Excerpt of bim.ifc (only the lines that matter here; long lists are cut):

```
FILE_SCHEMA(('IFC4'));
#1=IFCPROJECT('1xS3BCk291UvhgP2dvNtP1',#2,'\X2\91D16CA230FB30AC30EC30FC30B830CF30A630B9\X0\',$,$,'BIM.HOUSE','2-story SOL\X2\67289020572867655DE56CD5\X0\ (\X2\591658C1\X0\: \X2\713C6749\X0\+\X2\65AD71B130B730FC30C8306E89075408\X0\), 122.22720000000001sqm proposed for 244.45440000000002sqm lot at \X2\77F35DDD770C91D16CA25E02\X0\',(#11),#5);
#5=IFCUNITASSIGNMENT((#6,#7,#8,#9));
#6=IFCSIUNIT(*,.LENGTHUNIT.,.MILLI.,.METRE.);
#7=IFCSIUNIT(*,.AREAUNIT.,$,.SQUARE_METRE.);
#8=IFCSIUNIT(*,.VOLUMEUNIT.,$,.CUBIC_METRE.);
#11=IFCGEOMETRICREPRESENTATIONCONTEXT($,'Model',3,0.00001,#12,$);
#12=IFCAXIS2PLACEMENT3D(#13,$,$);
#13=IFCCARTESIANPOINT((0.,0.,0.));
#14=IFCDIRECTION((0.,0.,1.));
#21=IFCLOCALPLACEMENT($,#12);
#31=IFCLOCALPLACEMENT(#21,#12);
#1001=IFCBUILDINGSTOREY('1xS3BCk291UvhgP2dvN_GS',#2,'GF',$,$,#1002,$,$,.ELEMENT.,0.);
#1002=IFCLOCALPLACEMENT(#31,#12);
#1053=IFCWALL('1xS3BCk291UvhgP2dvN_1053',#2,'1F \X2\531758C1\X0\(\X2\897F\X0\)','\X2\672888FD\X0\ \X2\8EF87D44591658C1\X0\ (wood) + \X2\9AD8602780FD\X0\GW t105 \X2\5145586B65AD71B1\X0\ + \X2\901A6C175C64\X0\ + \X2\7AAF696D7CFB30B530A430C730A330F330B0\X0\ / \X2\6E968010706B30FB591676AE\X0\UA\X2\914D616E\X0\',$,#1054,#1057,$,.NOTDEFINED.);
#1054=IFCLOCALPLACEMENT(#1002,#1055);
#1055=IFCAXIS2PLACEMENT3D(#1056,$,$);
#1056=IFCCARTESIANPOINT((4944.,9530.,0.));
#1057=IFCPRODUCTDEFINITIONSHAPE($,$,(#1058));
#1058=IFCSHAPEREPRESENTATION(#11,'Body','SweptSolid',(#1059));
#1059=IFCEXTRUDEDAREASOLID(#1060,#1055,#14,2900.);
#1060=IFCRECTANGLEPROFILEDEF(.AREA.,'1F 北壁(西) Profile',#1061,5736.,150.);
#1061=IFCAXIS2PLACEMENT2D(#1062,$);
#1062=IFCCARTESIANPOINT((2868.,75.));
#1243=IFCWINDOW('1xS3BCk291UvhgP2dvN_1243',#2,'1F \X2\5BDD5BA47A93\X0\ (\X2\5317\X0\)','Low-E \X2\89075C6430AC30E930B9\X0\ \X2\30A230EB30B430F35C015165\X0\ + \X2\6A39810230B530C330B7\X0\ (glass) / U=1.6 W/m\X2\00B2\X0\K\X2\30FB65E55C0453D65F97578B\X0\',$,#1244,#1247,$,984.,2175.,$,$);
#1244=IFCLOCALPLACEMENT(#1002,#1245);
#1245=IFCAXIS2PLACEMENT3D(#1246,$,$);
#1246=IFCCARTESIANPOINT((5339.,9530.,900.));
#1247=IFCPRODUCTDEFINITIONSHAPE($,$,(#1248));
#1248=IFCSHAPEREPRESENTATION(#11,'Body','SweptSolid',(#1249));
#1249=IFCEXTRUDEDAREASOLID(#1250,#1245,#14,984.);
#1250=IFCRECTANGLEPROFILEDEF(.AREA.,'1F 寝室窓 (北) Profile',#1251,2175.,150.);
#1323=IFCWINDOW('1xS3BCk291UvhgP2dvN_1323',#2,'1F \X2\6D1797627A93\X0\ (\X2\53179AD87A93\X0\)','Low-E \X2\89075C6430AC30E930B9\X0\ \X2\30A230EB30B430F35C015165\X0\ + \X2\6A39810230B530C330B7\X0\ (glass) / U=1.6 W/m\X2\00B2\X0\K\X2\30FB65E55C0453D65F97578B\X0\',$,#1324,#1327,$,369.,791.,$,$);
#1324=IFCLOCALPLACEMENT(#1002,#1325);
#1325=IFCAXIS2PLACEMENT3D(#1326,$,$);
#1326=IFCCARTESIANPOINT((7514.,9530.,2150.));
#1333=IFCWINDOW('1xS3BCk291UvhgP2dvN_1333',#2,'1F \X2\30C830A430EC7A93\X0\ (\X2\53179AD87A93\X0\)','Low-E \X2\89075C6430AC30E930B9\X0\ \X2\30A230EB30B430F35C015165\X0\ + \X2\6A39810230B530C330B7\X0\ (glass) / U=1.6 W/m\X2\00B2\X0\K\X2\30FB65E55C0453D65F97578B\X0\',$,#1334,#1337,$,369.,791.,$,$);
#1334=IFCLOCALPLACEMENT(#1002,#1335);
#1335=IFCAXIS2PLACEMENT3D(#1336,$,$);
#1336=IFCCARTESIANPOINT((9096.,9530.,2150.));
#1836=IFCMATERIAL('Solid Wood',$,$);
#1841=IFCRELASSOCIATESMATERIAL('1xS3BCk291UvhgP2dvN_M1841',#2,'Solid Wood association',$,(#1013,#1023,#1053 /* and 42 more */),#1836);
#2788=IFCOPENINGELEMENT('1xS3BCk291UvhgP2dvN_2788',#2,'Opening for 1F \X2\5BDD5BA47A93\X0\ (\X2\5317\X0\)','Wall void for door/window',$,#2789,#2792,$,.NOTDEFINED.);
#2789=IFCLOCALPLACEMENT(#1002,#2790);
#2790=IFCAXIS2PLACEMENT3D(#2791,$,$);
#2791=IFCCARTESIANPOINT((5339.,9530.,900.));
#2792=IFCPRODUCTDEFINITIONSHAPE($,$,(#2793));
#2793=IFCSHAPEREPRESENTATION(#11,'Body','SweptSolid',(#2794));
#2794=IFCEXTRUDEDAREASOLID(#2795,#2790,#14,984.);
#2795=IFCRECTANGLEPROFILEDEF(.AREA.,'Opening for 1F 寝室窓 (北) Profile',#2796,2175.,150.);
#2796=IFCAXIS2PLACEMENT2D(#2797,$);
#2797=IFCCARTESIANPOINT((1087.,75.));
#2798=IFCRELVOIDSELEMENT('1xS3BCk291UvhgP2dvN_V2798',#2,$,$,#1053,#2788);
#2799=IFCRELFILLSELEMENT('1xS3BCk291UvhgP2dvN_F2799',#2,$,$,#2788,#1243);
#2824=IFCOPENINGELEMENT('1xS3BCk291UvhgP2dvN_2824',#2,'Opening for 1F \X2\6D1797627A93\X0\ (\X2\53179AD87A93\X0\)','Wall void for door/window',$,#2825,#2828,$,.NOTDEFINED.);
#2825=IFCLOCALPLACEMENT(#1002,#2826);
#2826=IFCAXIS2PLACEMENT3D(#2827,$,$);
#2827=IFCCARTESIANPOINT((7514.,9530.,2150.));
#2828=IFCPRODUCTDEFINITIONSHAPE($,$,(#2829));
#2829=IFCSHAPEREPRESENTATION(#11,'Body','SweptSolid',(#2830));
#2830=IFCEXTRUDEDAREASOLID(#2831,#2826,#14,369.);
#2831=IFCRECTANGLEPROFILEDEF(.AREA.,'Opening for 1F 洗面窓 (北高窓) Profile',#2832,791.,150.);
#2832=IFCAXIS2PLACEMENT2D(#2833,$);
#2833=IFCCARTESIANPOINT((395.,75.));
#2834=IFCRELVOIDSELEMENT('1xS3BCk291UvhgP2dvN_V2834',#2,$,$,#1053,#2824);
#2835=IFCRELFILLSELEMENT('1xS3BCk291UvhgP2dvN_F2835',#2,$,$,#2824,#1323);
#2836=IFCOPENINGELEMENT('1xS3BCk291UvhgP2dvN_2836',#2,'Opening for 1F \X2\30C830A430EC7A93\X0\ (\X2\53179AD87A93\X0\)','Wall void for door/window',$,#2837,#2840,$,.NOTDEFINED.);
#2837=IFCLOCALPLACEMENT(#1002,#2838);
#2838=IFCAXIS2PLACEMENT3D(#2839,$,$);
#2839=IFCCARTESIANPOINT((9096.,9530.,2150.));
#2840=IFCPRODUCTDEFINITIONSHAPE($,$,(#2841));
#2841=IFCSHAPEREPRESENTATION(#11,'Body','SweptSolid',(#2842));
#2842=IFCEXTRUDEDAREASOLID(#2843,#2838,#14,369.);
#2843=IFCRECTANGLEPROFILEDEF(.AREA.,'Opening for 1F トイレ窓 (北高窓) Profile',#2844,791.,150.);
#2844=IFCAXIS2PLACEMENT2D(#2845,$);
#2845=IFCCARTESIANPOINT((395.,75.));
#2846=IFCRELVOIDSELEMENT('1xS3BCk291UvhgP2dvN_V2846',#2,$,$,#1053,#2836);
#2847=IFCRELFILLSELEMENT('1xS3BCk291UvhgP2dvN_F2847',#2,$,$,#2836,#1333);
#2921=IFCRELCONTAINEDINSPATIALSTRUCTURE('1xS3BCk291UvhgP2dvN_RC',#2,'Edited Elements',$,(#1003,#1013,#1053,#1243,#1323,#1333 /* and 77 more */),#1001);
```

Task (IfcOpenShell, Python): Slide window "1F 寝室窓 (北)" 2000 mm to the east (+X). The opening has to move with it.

```python
import ifcopenshell
import ifcopenshell.api.geometry
import ifcopenshell.util.placement
import ifcopenshell.util.unit

model = ifcopenshell.open("bim.ifc")
unit_scale = ifcopenshell.util.unit.calculate_unit_scale(model)

window = model.by_guid("1xS3BCk291UvhgP2dvN_1243")
opening = window.FillsVoids[0].RelatingOpeningElement
wall = opening.VoidsElements[0].RelatingBuildingElement

wall_matrix = ifcopenshell.util.placement.get_local_placement(wall.ObjectPlacement)
shift = wall_matrix[:3, 0] * 2 / unit_scale
before = ifcopenshell.util.placement.get_local_placement(window.ObjectPlacement)[:3, 3].copy()

# The window is not placed relative to its opening, so move both.
for product in (opening, window):
    matrix = ifcopenshell.util.placement.get_local_placement(product.ObjectPlacement)
    matrix[:3, 3] += shift
    ifcopenshell.api.geometry.edit_object_placement(model, product=product, matrix=matrix, is_si=False)

after = ifcopenshell.util.placement.get_local_placement(window.ObjectPlacement)[:3, 3]
print("window moved by", (after - before).round(3) + 0.0)

model.write("bim_v2.ifc")
```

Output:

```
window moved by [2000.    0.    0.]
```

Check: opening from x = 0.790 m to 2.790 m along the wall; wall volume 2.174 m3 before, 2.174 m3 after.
